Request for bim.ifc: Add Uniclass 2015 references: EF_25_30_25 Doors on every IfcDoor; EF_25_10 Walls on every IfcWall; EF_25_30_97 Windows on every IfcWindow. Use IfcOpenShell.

First a look at what the model holds.

```python
import ifcopenshell

model = ifcopenshell.open("bim.ifc")
print(model.schema)
print("classifications:", [c.Name for c in model.by_type("IfcClassification")])
for ifc_class in ("IfcDoor", "IfcRoof", "IfcStair", "IfcWall", "IfcWindow"):
    print(ifc_class, len(model.by_type(ifc_class)))
```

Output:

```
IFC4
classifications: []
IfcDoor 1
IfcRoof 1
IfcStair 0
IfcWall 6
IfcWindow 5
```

```python
import ifcopenshell
import ifcopenshell.api.classification

model = ifcopenshell.open("bim.ifc")

system = ifcopenshell.api.classification.add_classification(model, classification="Uniclass 2015")

codes = {
    "IfcDoor": ("EF_25_30_25", "Doors"),
    "IfcWall": ("EF_25_10", "Walls"),
    "IfcWindow": ("EF_25_30_97", "Windows"),
}
for ifc_class, (code, name) in codes.items():
    products = model.by_type(ifc_class)
    ifcopenshell.api.classification.add_reference(
        model, products=products, classification=system, identification=code, name=name
    )
    print(code, len(products))

model.write("bim_rev.ifc")
```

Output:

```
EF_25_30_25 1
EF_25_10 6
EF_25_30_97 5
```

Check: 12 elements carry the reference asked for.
